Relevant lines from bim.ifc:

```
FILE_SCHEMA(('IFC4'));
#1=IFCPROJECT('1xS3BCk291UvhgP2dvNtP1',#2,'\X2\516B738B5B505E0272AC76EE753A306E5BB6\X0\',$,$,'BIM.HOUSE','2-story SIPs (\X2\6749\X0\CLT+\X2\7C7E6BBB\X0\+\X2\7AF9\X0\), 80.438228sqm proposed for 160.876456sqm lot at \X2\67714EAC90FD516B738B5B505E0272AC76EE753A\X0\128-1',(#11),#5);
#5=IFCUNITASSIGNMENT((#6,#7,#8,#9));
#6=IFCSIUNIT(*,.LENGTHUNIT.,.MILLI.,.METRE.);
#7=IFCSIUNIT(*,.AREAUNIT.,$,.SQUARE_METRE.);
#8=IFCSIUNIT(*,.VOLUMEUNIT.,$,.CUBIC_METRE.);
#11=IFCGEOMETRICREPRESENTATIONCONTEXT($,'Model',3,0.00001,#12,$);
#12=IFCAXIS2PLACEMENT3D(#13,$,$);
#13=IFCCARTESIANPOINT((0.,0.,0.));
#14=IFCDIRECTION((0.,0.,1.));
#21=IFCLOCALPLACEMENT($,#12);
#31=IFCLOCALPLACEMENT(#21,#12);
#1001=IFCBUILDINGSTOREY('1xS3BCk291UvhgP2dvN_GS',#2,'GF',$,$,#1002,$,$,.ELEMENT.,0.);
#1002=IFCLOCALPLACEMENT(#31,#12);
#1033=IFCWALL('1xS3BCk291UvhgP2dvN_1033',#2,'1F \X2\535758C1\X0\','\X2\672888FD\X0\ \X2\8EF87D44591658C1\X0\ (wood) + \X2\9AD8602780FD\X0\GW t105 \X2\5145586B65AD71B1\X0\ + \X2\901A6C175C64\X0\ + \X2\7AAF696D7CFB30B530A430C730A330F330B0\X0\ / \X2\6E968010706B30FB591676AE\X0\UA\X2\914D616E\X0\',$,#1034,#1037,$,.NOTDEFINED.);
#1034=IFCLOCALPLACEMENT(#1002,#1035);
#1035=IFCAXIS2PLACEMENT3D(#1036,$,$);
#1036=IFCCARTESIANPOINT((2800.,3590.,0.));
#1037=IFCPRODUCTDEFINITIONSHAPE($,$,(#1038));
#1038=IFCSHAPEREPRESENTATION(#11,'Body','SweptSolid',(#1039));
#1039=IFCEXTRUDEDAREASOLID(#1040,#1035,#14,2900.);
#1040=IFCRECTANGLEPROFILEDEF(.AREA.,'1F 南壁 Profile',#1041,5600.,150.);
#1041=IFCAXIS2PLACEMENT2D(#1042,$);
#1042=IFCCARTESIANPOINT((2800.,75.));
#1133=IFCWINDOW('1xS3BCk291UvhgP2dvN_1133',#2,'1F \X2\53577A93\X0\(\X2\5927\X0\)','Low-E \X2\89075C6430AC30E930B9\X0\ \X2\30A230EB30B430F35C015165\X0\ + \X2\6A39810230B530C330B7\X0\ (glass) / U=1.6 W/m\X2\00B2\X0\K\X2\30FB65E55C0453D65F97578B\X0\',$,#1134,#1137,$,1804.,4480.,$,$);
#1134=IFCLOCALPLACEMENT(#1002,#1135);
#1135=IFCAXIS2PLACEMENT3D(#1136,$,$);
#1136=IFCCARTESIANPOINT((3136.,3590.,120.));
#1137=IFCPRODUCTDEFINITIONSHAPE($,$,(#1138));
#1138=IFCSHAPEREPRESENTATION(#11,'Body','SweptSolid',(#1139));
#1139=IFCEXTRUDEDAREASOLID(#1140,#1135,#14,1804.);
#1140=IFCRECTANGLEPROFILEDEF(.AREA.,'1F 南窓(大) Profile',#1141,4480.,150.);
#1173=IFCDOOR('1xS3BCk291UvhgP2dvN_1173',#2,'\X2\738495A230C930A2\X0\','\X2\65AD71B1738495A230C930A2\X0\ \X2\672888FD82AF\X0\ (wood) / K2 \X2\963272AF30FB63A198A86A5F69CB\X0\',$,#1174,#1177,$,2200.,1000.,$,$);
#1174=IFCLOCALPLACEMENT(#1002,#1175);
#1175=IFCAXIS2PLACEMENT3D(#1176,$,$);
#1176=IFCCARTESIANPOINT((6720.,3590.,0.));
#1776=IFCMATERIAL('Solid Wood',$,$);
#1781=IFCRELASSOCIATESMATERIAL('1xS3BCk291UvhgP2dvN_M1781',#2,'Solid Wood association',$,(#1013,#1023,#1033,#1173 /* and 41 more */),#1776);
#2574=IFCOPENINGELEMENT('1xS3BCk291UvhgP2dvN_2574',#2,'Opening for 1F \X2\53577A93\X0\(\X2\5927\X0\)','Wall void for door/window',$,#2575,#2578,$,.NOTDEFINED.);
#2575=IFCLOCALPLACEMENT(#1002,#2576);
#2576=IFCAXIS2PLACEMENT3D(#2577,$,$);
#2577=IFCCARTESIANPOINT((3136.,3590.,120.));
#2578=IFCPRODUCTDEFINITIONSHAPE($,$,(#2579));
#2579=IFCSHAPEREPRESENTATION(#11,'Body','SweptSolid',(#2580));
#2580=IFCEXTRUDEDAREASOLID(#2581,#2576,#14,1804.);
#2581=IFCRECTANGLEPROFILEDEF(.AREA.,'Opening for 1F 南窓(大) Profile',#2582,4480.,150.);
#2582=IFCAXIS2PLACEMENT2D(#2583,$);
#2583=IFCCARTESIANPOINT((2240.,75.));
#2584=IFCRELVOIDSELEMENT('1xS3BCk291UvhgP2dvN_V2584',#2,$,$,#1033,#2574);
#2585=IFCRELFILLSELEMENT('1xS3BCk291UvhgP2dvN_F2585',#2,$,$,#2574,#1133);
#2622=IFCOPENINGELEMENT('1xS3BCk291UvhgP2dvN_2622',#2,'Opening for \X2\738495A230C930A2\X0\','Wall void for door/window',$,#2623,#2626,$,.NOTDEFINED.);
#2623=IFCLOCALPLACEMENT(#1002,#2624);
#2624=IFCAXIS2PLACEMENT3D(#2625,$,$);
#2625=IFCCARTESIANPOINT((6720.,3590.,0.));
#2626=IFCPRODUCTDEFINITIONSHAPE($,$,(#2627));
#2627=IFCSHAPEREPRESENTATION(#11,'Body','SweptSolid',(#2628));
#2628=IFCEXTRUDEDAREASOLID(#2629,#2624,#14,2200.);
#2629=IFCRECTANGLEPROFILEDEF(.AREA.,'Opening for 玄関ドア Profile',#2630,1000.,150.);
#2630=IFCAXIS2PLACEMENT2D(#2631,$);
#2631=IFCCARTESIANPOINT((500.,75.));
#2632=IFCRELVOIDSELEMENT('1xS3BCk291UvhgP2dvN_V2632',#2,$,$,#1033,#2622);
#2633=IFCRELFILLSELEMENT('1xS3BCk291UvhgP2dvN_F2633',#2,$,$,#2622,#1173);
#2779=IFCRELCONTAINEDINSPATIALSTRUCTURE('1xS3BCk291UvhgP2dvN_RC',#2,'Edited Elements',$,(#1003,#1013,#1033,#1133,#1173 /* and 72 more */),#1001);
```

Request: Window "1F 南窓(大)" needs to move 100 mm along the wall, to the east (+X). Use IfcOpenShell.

```python
import ifcopenshell
import ifcopenshell.api.geometry
import ifcopenshell.util.placement
import ifcopenshell.util.unit

model = ifcopenshell.open("bim.ifc")
unit_scale = ifcopenshell.util.unit.calculate_unit_scale(model)

window = model.by_guid("1xS3BCk291UvhgP2dvN_1133")
opening = window.FillsVoids[0].RelatingOpeningElement
wall = opening.VoidsElements[0].RelatingBuildingElement

wall_matrix = ifcopenshell.util.placement.get_local_placement(wall.ObjectPlacement)
shift = wall_matrix[:3, 0] * 0.1 / unit_scale
before = ifcopenshell.util.placement.get_local_placement(window.ObjectPlacement)[:3, 3].copy()

# The window is not placed relative to its opening, so move both.
for product in (opening, window):
    matrix = ifcopenshell.util.placement.get_local_placement(product.ObjectPlacement)
    matrix[:3, 3] += shift
    ifcopenshell.api.geometry.edit_object_placement(model, product=product, matrix=matrix, is_si=False)

after = ifcopenshell.util.placement.get_local_placement(window.ObjectPlacement)[:3, 3]
print("window moved by", (after - before).round(3) + 0.0)

model.write("bim_edited.ifc")
```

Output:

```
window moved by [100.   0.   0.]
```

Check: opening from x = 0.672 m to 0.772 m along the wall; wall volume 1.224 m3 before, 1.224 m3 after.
